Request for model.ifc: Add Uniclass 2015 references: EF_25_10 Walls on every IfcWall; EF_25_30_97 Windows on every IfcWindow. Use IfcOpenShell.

First a look at what the model holds.

```python
import ifcopenshell

model = ifcopenshell.open("model.ifc")
print(model.schema)
print("classifications:", [c.Name for c in model.by_type("IfcClassification")])
for ifc_class in ("IfcDoor", "IfcRoof", "IfcStair", "IfcWall", "IfcWindow"):
    print(ifc_class, len(model.by_type(ifc_class)))
```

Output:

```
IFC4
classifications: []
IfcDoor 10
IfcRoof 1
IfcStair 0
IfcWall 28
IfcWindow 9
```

```python
import ifcopenshell
import ifcopenshell.api.classification

model = ifcopenshell.open("model.ifc")

system = ifcopenshell.api.classification.add_classification(model, classification="Uniclass 2015")

codes = {
    "IfcWall": ("EF_25_10", "Walls"),
    "IfcWindow": ("EF_25_30_97", "Windows"),
}
for ifc_class, (code, name) in codes.items():
    products = model.by_type(ifc_class)
    ifcopenshell.api.classification.add_reference(
        model, products=products, classification=system, identification=code, name=name
    )
    print(code, len(products))

model.write("model_edited.ifc")
```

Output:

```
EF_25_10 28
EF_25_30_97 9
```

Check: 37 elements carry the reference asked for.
